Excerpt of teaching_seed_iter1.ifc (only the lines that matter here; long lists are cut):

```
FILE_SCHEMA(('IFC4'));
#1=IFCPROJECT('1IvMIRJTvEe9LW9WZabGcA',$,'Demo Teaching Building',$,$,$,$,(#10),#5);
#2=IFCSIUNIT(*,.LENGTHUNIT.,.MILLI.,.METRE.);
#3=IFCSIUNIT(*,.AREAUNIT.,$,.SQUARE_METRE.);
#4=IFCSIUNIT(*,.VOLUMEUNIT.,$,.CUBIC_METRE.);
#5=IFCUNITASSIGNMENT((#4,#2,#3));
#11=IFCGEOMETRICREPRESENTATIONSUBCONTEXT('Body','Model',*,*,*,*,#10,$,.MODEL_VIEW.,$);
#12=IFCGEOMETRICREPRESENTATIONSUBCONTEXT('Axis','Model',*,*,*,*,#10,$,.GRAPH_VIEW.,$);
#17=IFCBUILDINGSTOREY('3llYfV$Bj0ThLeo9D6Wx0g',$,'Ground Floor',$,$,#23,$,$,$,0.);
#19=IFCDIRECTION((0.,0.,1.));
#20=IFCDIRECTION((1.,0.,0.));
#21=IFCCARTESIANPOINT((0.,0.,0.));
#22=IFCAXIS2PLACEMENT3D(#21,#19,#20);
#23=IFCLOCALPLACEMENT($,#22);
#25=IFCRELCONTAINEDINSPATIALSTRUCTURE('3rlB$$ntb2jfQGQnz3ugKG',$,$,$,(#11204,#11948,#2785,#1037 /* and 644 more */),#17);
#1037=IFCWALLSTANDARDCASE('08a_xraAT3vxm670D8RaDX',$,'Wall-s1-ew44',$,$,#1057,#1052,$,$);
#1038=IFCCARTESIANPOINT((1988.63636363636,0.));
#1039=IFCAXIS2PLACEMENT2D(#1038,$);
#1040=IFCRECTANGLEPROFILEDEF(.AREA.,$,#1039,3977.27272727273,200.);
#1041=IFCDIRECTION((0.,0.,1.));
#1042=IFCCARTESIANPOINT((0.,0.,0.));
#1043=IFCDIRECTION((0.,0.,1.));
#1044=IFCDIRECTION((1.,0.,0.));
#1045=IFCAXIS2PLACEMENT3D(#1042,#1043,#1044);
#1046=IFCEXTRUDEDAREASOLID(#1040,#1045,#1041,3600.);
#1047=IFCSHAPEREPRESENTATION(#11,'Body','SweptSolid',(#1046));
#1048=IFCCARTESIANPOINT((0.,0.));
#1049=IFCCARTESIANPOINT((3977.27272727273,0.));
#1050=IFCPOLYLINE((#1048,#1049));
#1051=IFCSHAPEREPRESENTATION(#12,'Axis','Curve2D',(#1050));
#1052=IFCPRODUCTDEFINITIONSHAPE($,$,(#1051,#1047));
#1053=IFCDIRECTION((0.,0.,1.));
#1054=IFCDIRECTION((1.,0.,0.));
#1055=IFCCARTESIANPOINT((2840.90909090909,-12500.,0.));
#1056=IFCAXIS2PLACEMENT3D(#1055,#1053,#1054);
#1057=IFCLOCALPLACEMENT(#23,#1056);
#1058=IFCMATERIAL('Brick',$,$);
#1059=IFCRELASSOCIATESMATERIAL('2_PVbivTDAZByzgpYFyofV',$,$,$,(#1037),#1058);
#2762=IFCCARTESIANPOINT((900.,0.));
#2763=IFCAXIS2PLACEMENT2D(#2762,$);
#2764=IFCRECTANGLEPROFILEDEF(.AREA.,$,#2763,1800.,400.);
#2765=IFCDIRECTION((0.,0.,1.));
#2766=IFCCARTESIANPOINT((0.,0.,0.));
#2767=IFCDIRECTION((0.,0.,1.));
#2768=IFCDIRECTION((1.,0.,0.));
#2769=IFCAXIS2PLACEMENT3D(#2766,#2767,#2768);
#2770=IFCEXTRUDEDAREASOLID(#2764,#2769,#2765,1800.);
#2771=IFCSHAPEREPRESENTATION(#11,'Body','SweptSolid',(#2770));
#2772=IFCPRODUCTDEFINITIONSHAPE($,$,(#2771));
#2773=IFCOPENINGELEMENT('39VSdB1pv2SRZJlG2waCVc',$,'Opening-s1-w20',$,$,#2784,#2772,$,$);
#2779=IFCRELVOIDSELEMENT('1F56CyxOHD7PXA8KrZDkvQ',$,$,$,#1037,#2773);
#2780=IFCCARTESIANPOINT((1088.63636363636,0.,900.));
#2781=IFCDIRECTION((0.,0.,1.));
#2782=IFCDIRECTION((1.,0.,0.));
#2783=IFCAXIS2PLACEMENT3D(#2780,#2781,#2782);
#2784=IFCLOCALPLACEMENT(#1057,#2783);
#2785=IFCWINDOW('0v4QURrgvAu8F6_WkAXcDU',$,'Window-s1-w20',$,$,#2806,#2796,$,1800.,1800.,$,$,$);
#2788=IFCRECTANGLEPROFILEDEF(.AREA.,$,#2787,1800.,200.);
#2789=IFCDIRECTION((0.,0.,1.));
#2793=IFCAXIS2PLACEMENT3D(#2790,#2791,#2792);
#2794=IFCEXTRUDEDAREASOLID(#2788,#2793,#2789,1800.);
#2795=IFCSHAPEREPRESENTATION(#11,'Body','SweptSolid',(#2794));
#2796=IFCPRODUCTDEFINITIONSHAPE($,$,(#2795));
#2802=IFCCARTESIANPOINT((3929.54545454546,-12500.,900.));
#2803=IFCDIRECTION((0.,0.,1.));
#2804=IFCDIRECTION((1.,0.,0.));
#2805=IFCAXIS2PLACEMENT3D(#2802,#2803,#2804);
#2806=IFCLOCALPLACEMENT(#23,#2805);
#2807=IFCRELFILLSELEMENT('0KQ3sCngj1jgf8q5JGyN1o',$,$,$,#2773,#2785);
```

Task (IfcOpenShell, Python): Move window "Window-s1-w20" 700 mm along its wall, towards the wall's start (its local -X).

```python
import ifcopenshell
import ifcopenshell.api.geometry
import ifcopenshell.util.placement
import ifcopenshell.util.unit

model = ifcopenshell.open("teaching_seed_iter1.ifc")
unit_scale = ifcopenshell.util.unit.calculate_unit_scale(model)

window = model.by_id(2785)
opening = window.FillsVoids[0].RelatingOpeningElement
wall = opening.VoidsElements[0].RelatingBuildingElement

wall_matrix = ifcopenshell.util.placement.get_local_placement(wall.ObjectPlacement)
shift = wall_matrix[:3, 0] * -0.7 / unit_scale
before = ifcopenshell.util.placement.get_local_placement(window.ObjectPlacement)[:3, 3].copy()

# The window is not placed relative to its opening, so move both.
for product in (opening, window):
    matrix = ifcopenshell.util.placement.get_local_placement(product.ObjectPlacement)
    matrix[:3, 3] += shift
    ifcopenshell.api.geometry.edit_object_placement(model, product=product, matrix=matrix, is_si=False)

after = ifcopenshell.util.placement.get_local_placement(window.ObjectPlacement)[:3, 3]
print("window moved by", (after - before).round(3) + 0.0)

model.write("teaching_seed_iter1-out.ifc")
```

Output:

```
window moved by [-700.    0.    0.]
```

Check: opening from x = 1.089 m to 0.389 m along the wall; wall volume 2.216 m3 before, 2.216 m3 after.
